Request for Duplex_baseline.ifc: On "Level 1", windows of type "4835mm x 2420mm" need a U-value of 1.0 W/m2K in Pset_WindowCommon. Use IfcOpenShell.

First a look at what the model holds.

```python
import ifcopenshell
import ifcopenshell.util.element

model = ifcopenshell.open("Duplex_baseline.ifc")
print(model.schema)
storey = next(s for s in model.by_type("IfcBuildingStorey") if s.Name == "Level 1")
windows = [e for e in ifcopenshell.util.element.get_decomposition(storey) if e.is_a("IfcWindow")]
seen = {}
for e in windows:
    element_type = ifcopenshell.util.element.get_type(e)
    key = (element_type.Name if element_type != e and element_type else None, ifcopenshell.util.element.get_pset(e, "Pset_WindowCommon", "ThermalTransmittance"))
    seen[key] = seen.get(key, 0) + 1
for (name, value), count in sorted(seen.items(), key=str):
    print(count, "x", name, "|", value)
```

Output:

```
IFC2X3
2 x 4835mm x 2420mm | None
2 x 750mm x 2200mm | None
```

```python
import ifcopenshell
import ifcopenshell.api.pset
import ifcopenshell.util.element

model = ifcopenshell.open("Duplex_baseline.ifc")

storey = next(s for s in model.by_type("IfcBuildingStorey") if s.Name == "Level 1")
windows = [e for e in ifcopenshell.util.element.get_decomposition(storey) if e.is_a("IfcWindow")]

count = 0
for e in windows:
    element_type = ifcopenshell.util.element.get_type(e)
    if element_type in (None, e) or element_type.Name != "4835mm x 2420mm":
        continue
    # add_pset returns the element's existing set when there is one.
    pset = ifcopenshell.api.pset.add_pset(model, product=e, name="Pset_WindowCommon")
    ifcopenshell.api.pset.edit_pset(model, pset=pset, properties={"ThermalTransmittance": 1.0})
    count += 1

print(count, "windows updated")

model.write("Duplex_baseline_v2.ifc")
```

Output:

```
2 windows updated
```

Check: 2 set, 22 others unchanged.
